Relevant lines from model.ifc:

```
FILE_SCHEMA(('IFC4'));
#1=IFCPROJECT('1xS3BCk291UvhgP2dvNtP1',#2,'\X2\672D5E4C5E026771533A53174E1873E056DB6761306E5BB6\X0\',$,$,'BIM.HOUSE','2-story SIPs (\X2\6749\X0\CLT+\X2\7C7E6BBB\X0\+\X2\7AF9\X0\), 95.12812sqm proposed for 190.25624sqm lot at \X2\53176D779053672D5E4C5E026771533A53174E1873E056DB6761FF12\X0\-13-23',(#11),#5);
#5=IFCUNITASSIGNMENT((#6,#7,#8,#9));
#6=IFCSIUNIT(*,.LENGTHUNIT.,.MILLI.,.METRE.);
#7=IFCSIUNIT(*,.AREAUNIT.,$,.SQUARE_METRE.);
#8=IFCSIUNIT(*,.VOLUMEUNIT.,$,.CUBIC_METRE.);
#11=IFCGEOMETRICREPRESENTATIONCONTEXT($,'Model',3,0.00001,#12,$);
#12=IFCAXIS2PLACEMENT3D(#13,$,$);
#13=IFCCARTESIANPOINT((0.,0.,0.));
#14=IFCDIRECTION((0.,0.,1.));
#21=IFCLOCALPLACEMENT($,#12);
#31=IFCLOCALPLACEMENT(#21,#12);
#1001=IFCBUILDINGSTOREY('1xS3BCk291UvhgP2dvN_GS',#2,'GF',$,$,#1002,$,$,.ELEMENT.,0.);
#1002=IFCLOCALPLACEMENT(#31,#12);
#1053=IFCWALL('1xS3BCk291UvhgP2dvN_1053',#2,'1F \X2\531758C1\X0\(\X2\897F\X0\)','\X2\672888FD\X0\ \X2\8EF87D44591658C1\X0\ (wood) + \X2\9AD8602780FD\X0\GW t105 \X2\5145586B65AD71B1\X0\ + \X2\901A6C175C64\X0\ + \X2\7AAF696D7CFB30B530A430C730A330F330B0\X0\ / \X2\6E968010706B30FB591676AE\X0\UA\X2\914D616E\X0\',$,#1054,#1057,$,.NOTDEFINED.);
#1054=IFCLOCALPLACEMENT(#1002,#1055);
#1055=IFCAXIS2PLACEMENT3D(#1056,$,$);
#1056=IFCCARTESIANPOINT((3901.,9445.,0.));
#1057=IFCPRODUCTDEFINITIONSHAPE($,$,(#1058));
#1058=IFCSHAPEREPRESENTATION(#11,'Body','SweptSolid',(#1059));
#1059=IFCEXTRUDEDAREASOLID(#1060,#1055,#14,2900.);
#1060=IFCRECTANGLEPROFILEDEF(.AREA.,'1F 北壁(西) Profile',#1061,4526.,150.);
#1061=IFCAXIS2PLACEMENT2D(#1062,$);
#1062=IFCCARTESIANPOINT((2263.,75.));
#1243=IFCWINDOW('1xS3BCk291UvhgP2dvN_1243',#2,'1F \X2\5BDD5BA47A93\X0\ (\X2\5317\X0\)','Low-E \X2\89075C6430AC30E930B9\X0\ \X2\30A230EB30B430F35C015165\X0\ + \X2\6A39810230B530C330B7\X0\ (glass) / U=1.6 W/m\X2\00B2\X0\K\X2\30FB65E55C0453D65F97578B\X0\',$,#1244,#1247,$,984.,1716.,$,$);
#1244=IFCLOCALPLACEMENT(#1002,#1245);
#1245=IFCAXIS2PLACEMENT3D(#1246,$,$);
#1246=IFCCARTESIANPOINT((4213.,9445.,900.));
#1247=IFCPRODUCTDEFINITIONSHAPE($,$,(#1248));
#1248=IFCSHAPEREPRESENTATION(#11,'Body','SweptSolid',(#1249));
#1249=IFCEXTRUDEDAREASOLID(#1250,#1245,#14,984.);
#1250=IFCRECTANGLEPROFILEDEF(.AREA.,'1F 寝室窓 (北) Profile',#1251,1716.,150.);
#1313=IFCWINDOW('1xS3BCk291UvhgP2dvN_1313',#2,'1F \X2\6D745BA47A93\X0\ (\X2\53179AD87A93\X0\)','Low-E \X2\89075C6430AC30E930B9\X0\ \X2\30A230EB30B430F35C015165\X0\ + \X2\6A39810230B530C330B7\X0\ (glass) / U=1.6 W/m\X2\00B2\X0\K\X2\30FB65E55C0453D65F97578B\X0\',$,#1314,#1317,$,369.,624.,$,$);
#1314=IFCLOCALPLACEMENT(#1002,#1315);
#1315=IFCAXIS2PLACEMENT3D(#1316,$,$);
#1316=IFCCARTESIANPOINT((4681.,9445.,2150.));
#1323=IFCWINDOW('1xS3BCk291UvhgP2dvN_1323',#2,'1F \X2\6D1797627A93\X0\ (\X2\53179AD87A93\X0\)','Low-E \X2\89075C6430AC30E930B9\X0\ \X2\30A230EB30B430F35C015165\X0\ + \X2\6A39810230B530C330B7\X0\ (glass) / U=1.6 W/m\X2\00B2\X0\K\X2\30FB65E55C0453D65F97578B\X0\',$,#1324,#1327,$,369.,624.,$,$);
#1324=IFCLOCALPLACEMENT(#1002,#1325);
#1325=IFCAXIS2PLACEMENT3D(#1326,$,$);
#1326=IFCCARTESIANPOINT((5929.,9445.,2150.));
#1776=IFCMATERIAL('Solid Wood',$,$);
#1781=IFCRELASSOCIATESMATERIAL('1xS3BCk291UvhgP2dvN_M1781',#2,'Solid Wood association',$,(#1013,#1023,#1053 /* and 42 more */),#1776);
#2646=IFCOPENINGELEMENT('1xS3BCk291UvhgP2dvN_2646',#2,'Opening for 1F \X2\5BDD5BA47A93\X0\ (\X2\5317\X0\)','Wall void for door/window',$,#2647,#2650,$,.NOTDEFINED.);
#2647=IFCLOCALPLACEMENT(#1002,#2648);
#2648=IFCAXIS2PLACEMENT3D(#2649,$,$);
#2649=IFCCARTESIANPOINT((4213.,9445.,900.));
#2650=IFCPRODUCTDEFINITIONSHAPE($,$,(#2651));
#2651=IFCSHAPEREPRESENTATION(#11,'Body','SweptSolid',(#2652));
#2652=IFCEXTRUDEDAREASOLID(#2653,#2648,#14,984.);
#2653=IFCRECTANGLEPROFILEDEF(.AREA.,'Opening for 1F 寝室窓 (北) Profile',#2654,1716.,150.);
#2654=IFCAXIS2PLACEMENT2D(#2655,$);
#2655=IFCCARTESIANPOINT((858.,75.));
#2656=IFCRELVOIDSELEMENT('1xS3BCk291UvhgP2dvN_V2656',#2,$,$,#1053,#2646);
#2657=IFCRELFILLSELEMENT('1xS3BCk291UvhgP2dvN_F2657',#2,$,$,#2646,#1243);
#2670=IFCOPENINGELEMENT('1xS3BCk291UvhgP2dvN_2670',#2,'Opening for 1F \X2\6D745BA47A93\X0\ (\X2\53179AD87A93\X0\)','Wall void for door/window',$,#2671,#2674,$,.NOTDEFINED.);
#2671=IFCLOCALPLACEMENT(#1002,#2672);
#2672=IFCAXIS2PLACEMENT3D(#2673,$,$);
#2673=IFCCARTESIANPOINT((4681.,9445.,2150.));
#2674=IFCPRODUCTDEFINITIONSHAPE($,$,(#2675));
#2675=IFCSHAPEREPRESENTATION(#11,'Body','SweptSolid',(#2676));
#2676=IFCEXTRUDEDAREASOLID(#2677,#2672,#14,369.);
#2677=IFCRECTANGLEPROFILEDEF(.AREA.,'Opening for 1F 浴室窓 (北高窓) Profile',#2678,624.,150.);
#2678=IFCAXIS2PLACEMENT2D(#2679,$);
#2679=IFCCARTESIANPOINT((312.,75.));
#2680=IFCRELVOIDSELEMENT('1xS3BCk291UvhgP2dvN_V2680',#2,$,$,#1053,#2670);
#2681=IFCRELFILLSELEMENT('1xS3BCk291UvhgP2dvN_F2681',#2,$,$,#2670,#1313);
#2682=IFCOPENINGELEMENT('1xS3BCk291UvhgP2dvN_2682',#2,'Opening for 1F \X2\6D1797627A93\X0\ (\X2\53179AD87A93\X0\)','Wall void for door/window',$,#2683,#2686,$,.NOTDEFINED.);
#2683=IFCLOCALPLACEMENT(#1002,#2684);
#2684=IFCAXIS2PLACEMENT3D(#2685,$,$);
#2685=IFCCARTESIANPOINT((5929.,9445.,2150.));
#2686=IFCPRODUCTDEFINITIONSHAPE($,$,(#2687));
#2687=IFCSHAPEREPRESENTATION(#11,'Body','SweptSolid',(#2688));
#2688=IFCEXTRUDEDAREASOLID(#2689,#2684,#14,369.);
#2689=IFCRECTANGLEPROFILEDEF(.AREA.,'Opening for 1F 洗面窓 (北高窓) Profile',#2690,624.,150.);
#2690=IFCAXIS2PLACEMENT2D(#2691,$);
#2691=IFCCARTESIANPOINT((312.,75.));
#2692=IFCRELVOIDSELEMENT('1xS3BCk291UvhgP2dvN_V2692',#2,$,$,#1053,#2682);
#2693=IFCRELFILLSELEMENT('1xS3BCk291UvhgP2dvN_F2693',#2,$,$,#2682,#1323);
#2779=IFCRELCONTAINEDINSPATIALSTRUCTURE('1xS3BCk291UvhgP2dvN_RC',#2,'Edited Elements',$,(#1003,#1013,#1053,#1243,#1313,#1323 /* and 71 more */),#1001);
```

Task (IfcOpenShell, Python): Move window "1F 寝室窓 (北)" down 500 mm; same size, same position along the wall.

```python
import numpy as np
import ifcopenshell
import ifcopenshell.api.geometry
import ifcopenshell.util.placement
import ifcopenshell.util.unit

model = ifcopenshell.open("model.ifc")
unit_scale = ifcopenshell.util.unit.calculate_unit_scale(model)

window = model.by_guid("1xS3BCk291UvhgP2dvN_1243")
opening = window.FillsVoids[0].RelatingOpeningElement
dz = -500.0

shift = np.array([0.0, 0.0, dz])
# The window is not placed relative to its opening, so move both.
for product in (opening, window):
    matrix = ifcopenshell.util.placement.get_local_placement(product.ObjectPlacement)
    matrix[:3, 3] += shift
    ifcopenshell.api.geometry.edit_object_placement(model, product=product, matrix=matrix, is_si=False)

print(f"moved by {dz * unit_scale:+.3f} m")

model.write("model-out.ifc")
```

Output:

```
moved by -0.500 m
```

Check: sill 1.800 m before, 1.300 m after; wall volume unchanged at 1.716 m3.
